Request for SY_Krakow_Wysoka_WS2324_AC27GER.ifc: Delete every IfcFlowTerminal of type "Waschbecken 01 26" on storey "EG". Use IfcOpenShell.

First a look at what the model holds.

```python
import ifcopenshell
import ifcopenshell.util.element

model = ifcopenshell.open("SY_Krakow_Wysoka_WS2324_AC27GER.ifc")
print(model.schema)
storey = next(s for s in model.by_type("IfcBuildingStorey") if s.Name == "EG")
terminals = [e for e in ifcopenshell.util.element.get_decomposition(storey) if e.is_a("IfcFlowTerminal")]
seen = {}
for e in terminals:
    element_type = ifcopenshell.util.element.get_type(e)
    name = element_type.Name if element_type not in (None, e) else None
    seen[name] = seen.get(name, 0) + 1
for name, count in sorted(seen.items(), key=str):
    print(count, "x", name)
```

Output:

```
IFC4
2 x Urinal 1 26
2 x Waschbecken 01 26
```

```python
import ifcopenshell
import ifcopenshell.api.root
import ifcopenshell.util.element

model = ifcopenshell.open("SY_Krakow_Wysoka_WS2324_AC27GER.ifc")

storey = next(s for s in model.by_type("IfcBuildingStorey") if s.Name == "EG")
terminals = [e for e in ifcopenshell.util.element.get_decomposition(storey) if e.is_a("IfcFlowTerminal")]
targets = [e for e in terminals if (t := ifcopenshell.util.element.get_type(e)) not in (None, e) and t.Name == "Waschbecken 01 26"]

for e in targets:
    ifcopenshell.api.root.remove_product(model, product=e)
print(len(targets), "removed")

model.write("SY_Krakow_Wysoka_WS2324_AC27GER-out.ifc")
```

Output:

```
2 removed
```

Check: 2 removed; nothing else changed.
